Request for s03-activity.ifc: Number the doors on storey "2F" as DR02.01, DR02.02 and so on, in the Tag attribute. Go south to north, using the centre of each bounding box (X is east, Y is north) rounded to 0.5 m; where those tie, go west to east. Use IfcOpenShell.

First a look at what the model holds.

```python
import ifcopenshell
import ifcopenshell.util.element
import ifcopenshell.util.placement

model = ifcopenshell.open("s03-activity.ifc")
print(model.schema)
storey = next(s for s in model.by_type("IfcBuildingStorey") if s.Name == "2F")
doors = [e for e in ifcopenshell.util.element.get_decomposition(storey) if e.is_a("IfcDoor")]
for e in sorted(doors, key=lambda e: e.id()):
    origin = ifcopenshell.util.placement.get_local_placement(e.ObjectPlacement)[:3, 3]
    print(e.id(), e.Tag, e.Name, origin.round(2) + 0.0, sep=" | ")
```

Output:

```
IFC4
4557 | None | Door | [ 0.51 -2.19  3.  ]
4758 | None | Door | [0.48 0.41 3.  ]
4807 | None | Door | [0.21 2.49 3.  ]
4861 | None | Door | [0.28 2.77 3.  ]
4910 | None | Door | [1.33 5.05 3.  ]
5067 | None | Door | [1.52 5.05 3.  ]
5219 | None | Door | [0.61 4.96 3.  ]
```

```python
import ifcopenshell
import ifcopenshell.geom
import ifcopenshell.util.element
import ifcopenshell.util.shape

model = ifcopenshell.open("s03-activity.ifc")
settings = ifcopenshell.geom.settings()
settings.set("use-world-coords", True)


def centre(element):
    shape = ifcopenshell.geom.create_shape(settings, element)
    return ifcopenshell.util.shape.get_bbox_centroid(shape.geometry)


storey = next(s for s in model.by_type("IfcBuildingStorey") if s.Name == "2F")
doors = [e for e in ifcopenshell.util.element.get_decomposition(storey) if e.is_a("IfcDoor")]

# Insertion points can sit at a corner or the storey origin, so sort by the geometry (in metres).
centres = {e: centre(e) for e in doors}
doors.sort(key=lambda e: (round(centres[e][1] / 0.5), centres[e][0]))

for i, e in enumerate(doors, start=1):
    number = f"DR02.{i:02d}"
    e.Tag = number
    print(e.id(), number)

model.write("s03-activity-out.ifc")
```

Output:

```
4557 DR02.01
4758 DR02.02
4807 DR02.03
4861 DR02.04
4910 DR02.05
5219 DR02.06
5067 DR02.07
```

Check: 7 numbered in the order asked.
